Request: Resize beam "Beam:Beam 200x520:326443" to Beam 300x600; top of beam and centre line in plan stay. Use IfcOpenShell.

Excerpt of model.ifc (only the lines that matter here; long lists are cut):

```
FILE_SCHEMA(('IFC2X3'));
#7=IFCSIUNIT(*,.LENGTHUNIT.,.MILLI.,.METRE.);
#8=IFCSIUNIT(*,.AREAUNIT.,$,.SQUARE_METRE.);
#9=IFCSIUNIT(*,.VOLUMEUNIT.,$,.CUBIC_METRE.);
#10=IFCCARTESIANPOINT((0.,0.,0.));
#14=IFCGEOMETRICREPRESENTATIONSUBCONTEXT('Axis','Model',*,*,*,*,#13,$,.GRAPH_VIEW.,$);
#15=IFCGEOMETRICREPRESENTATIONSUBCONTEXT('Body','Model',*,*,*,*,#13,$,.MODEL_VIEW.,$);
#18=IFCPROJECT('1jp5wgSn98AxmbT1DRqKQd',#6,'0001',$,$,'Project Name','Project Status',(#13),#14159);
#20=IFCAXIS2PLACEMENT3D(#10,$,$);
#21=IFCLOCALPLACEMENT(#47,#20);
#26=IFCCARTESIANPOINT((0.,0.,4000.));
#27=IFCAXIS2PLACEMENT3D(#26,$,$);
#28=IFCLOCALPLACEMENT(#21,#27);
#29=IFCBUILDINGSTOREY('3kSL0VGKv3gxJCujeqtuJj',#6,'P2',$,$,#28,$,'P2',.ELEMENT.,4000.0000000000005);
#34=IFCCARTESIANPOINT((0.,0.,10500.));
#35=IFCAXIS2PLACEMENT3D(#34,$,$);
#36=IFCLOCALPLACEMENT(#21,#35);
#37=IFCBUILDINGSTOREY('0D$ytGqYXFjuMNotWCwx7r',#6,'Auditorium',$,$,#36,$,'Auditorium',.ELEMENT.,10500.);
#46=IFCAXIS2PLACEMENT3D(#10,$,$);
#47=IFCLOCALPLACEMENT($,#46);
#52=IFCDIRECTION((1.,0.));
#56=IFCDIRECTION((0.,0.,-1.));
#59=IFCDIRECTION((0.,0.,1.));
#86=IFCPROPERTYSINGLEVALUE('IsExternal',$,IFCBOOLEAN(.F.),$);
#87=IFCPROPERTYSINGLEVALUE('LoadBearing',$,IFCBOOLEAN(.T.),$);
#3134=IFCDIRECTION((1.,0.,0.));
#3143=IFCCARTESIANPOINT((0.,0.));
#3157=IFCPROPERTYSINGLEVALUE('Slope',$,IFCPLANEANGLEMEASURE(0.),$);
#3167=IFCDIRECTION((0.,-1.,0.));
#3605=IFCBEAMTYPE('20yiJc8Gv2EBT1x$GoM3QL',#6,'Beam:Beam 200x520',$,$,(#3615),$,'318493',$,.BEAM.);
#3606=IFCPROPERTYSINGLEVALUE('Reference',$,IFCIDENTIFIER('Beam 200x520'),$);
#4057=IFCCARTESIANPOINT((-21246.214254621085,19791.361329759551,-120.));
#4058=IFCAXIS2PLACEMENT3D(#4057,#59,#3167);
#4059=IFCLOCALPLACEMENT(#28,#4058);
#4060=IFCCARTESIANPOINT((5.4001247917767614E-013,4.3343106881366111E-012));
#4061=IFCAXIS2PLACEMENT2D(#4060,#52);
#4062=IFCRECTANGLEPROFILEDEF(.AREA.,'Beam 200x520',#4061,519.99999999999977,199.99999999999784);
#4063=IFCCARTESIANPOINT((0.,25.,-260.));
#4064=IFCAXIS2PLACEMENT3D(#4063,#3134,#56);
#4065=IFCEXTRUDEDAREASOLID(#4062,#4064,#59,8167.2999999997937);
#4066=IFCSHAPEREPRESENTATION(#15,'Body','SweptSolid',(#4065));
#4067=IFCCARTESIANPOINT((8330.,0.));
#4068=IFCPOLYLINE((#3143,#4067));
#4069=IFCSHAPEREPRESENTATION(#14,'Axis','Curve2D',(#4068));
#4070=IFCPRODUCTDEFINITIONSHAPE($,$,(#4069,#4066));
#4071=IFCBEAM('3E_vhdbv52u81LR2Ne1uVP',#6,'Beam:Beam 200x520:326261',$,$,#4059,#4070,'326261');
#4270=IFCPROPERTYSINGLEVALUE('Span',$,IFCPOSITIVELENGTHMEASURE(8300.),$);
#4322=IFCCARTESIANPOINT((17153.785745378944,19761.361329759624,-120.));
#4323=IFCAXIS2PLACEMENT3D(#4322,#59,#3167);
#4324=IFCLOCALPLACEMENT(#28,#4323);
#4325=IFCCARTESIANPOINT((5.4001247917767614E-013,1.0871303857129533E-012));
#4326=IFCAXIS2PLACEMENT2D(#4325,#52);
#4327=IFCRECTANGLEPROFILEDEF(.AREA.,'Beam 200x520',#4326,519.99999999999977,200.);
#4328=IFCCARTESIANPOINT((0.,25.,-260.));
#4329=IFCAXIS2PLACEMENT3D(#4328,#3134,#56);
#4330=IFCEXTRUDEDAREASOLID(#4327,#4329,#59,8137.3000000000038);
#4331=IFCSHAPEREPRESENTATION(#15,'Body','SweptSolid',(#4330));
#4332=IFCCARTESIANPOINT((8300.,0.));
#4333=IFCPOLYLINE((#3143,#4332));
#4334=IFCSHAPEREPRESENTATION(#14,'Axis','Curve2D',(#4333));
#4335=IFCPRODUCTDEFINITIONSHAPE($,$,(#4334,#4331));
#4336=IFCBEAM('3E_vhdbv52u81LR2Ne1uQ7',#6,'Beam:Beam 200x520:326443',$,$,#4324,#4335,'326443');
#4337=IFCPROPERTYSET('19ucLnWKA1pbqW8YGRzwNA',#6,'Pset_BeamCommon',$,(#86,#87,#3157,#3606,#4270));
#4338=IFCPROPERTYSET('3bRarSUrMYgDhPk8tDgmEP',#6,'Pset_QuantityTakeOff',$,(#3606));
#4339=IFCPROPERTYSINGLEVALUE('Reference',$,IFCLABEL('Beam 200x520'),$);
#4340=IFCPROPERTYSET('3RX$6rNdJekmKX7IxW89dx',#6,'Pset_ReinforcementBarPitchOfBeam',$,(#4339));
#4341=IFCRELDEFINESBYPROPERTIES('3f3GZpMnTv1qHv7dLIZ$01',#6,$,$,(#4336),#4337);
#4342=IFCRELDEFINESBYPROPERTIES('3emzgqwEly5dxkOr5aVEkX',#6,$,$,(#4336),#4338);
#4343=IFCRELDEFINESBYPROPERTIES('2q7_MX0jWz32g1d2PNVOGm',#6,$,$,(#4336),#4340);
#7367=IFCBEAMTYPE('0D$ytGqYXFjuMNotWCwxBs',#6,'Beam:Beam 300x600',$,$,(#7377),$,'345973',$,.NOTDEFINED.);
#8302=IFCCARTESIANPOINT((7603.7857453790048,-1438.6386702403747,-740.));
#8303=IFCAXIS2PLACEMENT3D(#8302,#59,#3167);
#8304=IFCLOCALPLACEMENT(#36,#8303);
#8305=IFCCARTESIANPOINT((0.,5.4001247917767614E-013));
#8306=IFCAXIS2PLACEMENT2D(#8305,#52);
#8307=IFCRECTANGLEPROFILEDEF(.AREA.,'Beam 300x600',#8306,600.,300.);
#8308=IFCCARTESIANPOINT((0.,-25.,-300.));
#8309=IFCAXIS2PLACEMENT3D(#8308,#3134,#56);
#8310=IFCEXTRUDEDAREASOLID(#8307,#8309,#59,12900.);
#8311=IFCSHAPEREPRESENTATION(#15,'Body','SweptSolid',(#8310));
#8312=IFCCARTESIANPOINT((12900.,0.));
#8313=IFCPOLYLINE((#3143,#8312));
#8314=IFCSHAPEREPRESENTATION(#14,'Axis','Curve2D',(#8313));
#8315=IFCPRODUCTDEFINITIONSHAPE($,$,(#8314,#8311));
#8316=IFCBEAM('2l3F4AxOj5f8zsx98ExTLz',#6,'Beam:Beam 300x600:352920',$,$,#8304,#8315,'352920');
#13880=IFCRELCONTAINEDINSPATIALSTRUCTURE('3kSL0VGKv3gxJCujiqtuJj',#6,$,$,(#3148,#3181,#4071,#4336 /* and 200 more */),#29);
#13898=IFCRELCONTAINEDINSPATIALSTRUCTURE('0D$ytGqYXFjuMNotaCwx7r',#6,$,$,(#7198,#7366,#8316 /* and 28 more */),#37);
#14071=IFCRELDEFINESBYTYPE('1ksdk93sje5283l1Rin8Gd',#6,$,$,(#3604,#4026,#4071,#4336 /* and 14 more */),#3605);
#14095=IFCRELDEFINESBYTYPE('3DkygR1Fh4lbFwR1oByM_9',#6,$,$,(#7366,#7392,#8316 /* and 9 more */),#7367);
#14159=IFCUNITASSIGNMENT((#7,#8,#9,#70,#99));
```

```python
import ifcopenshell
import ifcopenshell.api.pset
import ifcopenshell.api.type
import ifcopenshell.util.element
import ifcopenshell.util.representation

model = ifcopenshell.open("model.ifc")

member = model.by_guid("3E_vhdbv52u81LR2Ne1uQ7")
source = next(p for p in model.by_type("IfcRectangleProfileDef") if p.ProfileName == "Beam 300x600")

body = ifcopenshell.util.representation.get_representation(member, "Model", "Body")
solid = body.Items[0]
old_profile = solid.SweptArea

# Copy the section's sizes but keep this member's own profile position.
profile = ifcopenshell.util.element.copy(model, source)
# Profiles are centred, so shift by half the change in depth to hold the top.
shift = (old_profile.XDim - profile.XDim) / 2
x, y = old_profile.Position.Location.Coordinates
up = (-1.0, 0.0)  # upwards, in the solid's own plane
location = model.createIfcCartesianPoint((x + up[0] * shift, y + up[1] * shift))
profile.Position = model.createIfcAxis2Placement2D(location, old_profile.Position.RefDirection)
solid.SweptArea = profile
if not model.get_total_inverses(old_profile):
    ifcopenshell.util.element.remove_deep2(model, old_profile)

new_type = model.by_guid("0D$ytGqYXFjuMNotWCwxBs")
ifcopenshell.api.type.assign_type(
    model, related_objects=[member], relating_type=new_type, should_map_representations=False
)
member.Name = member.Name.replace("Beam 200x520", "Beam 300x600")
pset = model.by_id(ifcopenshell.util.element.get_pset(member, "Pset_BeamCommon", should_inherit=False)["id"])
ifcopenshell.api.pset.edit_pset(model, pset=pset, properties={"Reference": "Beam 300x600"})
pset = model.by_id(ifcopenshell.util.element.get_pset(member, "Pset_QuantityTakeOff", should_inherit=False)["id"])
ifcopenshell.api.pset.edit_pset(model, pset=pset, properties={"Reference": "Beam 300x600"})
pset = model.by_id(ifcopenshell.util.element.get_pset(member, "Pset_ReinforcementBarPitchOfBeam", should_inherit=False)["id"])
ifcopenshell.api.pset.edit_pset(model, pset=pset, properties={"Reference": "Beam 300x600"})

print(solid.SweptArea)

model.write("model_updated.ifc")
```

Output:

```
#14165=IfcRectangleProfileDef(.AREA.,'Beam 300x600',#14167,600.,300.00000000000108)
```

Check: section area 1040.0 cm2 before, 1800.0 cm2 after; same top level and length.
